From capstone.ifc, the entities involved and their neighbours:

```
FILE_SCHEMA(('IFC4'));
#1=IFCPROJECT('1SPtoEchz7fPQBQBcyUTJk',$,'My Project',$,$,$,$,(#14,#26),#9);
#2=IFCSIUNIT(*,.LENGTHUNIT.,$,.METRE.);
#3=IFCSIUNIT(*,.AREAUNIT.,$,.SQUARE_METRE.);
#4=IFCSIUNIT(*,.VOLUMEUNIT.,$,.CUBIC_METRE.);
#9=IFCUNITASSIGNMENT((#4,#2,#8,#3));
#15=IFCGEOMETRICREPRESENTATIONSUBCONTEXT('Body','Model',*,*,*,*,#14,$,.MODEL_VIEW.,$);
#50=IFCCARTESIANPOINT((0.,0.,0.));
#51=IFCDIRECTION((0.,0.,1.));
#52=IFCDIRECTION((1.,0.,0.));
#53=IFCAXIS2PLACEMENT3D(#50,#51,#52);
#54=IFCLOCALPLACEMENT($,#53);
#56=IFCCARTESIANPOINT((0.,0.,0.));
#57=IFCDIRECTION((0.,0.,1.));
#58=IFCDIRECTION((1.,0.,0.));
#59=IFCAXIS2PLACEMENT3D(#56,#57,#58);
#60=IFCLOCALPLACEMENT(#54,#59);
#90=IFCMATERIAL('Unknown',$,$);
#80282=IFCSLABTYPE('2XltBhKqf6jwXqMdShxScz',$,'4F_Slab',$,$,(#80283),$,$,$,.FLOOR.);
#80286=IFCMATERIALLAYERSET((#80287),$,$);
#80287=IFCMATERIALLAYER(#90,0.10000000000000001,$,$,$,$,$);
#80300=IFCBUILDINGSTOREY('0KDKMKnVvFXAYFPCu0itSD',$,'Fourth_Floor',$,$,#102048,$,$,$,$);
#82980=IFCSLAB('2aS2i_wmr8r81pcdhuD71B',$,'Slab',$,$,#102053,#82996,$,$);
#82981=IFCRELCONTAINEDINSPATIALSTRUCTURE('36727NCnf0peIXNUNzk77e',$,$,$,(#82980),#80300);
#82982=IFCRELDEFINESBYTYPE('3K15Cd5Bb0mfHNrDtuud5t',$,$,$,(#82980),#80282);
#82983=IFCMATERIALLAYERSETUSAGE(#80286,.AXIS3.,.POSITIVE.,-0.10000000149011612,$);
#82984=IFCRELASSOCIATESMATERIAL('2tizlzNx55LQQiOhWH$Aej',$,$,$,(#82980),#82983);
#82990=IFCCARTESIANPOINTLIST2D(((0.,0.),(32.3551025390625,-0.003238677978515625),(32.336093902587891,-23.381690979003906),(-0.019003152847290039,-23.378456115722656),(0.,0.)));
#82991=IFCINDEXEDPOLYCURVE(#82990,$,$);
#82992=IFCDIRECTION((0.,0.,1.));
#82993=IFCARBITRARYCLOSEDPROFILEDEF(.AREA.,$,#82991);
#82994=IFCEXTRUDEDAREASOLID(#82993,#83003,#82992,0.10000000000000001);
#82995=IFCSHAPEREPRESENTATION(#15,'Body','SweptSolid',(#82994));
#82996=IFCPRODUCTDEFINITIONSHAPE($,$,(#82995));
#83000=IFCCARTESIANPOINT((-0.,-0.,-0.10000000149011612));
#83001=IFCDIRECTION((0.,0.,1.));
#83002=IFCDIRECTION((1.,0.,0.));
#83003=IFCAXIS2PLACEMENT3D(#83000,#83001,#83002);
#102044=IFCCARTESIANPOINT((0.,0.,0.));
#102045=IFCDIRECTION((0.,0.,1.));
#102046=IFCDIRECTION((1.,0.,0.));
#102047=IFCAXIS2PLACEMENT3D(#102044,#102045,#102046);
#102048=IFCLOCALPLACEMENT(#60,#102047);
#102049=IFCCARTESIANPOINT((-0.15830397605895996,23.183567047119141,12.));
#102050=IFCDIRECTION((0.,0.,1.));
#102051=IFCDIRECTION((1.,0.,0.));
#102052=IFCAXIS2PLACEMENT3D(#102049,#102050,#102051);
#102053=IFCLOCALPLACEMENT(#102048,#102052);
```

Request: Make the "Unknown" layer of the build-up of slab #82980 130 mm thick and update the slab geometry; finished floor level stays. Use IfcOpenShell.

```python
import ifcopenshell
import ifcopenshell.util.element
import ifcopenshell.util.representation

model = ifcopenshell.open("capstone.ifc")

layer_set = model.by_id(80286)
layer = next(l for l in layer_set.MaterialLayers if l.Material and l.Material.Name == "Unknown")
change = 0.13 - layer.LayerThickness
layer.LayerThickness += change

# Geometry does not follow the layer set by itself.
slabs = [e for e in ifcopenshell.util.element.get_elements_by_material(model, layer_set) if e.is_a("IfcSlab")]
for slab in sorted(slabs, key=lambda e: e.id()):
    body = ifcopenshell.util.representation.get_representation(slab, "Model", "Body")
    solid = body.Items[0]
    old_depth = solid.Depth
    solid.Depth += change
    # Extruded upwards: lower the start of the extrusion so the top stays.
    x, y, z = solid.Position.Location.Coordinates
    solid.Position.Location = model.createIfcCartesianPoint((x, y, z - change))
    print(slab.id(), f"{old_depth:g} -> {solid.Depth:g}")

# The layers are counted up from the underside, which has moved.
for usage in {ifcopenshell.util.element.get_material(slab) for slab in slabs}:
    usage.OffsetFromReferenceLine -= change

model.write("capstone-out.ifc")
```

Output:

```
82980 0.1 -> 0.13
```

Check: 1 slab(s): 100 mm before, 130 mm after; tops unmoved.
